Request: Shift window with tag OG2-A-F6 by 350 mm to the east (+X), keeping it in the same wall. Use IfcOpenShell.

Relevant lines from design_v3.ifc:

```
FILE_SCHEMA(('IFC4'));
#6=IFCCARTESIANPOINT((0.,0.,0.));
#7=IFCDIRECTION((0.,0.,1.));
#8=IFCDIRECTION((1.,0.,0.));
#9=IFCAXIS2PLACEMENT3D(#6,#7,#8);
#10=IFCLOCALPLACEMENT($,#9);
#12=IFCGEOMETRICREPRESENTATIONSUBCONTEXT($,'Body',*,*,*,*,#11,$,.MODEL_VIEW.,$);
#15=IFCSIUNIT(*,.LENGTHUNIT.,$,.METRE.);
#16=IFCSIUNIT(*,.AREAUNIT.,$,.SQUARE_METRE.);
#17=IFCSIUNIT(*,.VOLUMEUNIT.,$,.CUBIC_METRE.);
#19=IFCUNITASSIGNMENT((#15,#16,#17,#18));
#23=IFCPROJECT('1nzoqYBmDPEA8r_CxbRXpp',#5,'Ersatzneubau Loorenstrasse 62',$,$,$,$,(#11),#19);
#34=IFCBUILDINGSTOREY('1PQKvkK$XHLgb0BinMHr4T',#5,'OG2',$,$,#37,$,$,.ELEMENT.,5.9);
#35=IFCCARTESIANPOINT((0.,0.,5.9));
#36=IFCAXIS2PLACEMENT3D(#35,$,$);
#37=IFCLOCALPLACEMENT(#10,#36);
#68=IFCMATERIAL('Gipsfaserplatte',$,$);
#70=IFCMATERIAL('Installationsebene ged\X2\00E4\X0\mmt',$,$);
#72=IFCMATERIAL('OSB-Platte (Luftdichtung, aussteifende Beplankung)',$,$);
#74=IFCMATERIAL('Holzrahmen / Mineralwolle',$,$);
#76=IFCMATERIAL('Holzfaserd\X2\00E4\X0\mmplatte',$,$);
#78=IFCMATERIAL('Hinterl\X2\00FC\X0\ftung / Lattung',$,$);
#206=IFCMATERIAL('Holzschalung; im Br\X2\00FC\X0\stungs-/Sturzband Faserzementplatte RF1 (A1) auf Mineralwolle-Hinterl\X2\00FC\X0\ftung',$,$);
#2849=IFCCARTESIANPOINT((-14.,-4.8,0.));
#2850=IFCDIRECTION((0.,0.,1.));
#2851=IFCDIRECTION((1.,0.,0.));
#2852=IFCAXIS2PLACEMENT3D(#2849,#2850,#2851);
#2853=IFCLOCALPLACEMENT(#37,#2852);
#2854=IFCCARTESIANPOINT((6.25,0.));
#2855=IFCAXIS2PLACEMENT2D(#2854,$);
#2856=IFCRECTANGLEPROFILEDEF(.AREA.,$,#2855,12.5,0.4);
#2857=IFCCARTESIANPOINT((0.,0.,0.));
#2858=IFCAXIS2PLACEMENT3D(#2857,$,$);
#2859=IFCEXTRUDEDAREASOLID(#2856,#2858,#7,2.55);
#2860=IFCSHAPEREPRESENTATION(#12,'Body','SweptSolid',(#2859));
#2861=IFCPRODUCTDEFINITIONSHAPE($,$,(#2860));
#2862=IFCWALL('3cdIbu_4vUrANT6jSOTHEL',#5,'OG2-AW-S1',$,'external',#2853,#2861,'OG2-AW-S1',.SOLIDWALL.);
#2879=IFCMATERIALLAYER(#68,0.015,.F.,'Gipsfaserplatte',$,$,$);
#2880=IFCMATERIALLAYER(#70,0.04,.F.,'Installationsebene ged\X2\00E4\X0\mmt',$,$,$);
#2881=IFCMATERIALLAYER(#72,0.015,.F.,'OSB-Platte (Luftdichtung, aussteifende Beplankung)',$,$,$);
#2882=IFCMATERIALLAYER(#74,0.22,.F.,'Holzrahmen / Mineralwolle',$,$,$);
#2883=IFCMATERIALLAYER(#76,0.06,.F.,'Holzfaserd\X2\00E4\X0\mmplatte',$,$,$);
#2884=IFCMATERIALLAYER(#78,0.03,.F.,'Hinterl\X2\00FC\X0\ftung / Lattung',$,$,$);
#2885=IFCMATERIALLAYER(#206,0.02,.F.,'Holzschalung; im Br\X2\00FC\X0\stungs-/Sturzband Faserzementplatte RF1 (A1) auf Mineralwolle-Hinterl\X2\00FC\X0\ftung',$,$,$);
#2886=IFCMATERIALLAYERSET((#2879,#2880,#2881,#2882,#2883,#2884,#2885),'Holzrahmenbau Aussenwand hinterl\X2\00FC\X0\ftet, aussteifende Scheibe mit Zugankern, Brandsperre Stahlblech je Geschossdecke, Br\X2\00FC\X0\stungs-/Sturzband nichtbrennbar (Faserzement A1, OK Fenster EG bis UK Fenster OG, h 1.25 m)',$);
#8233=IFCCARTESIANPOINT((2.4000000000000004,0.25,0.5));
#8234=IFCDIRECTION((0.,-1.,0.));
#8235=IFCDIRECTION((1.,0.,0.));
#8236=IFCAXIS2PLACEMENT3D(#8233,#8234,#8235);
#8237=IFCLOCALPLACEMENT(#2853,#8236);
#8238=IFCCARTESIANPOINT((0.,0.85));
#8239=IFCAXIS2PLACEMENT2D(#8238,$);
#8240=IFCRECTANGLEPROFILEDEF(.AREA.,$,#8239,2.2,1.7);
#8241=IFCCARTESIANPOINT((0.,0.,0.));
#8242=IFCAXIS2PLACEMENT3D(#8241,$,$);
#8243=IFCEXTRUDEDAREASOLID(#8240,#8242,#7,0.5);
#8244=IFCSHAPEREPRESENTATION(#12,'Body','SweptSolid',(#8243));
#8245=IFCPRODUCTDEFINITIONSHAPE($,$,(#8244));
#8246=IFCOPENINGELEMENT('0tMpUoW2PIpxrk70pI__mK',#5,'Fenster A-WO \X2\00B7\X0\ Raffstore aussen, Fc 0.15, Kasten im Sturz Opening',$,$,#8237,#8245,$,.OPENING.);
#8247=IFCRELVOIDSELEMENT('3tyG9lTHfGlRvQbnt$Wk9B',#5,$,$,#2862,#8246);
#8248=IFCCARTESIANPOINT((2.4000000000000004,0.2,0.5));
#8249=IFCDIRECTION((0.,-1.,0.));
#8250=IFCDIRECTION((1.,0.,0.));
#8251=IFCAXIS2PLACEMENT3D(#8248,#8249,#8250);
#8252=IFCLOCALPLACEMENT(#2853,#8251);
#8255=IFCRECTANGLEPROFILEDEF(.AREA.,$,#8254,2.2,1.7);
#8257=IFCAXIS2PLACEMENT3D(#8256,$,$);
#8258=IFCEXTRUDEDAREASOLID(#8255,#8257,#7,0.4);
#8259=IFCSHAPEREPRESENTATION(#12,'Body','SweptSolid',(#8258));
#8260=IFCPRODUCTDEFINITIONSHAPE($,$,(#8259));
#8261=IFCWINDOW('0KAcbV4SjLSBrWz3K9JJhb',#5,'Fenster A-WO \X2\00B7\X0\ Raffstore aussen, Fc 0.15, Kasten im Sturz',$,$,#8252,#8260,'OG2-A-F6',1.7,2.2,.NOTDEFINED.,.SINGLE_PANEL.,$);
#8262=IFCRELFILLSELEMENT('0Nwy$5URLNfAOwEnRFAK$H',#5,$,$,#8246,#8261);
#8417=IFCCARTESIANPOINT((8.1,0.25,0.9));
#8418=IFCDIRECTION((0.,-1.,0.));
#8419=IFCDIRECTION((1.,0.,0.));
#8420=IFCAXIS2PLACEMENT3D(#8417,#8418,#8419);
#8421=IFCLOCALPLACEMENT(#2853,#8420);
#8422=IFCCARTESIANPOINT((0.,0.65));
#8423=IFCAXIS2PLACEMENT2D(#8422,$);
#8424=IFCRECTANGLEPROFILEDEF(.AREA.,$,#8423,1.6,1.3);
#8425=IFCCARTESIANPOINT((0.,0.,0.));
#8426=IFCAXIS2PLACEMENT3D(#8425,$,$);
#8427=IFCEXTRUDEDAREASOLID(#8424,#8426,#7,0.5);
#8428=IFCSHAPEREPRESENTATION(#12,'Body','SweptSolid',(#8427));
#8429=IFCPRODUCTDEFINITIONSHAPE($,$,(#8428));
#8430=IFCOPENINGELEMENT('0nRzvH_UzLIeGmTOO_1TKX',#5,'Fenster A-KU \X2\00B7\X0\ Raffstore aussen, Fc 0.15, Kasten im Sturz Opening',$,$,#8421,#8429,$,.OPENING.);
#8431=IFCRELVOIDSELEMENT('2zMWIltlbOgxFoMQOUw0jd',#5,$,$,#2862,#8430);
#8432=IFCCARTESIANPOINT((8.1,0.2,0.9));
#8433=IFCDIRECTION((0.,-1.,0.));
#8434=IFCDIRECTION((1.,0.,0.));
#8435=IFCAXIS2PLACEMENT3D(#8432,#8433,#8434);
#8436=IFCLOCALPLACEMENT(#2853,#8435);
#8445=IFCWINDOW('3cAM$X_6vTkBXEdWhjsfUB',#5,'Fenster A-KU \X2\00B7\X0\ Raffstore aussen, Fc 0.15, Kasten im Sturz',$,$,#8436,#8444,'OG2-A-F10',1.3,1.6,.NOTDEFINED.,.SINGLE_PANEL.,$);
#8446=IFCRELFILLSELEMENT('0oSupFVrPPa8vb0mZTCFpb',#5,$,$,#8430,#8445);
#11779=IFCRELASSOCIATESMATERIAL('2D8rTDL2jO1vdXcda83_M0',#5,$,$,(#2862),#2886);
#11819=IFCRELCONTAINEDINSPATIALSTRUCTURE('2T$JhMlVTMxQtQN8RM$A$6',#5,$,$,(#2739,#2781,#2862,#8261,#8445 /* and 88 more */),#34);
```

```python
import ifcopenshell
import ifcopenshell.api.geometry
import ifcopenshell.util.placement

model = ifcopenshell.open("design_v3.ifc")

window = model.by_guid("0KAcbV4SjLSBrWz3K9JJhb")
opening = window.FillsVoids[0].RelatingOpeningElement
wall = opening.VoidsElements[0].RelatingBuildingElement

wall_matrix = ifcopenshell.util.placement.get_local_placement(wall.ObjectPlacement)
shift = wall_matrix[:3, 0] * 0.35
before = ifcopenshell.util.placement.get_local_placement(window.ObjectPlacement)[:3, 3].copy()

# The window is not placed relative to its opening, so move both.
for product in (opening, window):
    matrix = ifcopenshell.util.placement.get_local_placement(product.ObjectPlacement)
    matrix[:3, 3] += shift
    ifcopenshell.api.geometry.edit_object_placement(model, product=product, matrix=matrix, is_si=False)

after = ifcopenshell.util.placement.get_local_placement(window.ObjectPlacement)[:3, 3]
print("window moved by", (after - before).round(3) + 0.0)

model.write("design_v3_v2.ifc")
```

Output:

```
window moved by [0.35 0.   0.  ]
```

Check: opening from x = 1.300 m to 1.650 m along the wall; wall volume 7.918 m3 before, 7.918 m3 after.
